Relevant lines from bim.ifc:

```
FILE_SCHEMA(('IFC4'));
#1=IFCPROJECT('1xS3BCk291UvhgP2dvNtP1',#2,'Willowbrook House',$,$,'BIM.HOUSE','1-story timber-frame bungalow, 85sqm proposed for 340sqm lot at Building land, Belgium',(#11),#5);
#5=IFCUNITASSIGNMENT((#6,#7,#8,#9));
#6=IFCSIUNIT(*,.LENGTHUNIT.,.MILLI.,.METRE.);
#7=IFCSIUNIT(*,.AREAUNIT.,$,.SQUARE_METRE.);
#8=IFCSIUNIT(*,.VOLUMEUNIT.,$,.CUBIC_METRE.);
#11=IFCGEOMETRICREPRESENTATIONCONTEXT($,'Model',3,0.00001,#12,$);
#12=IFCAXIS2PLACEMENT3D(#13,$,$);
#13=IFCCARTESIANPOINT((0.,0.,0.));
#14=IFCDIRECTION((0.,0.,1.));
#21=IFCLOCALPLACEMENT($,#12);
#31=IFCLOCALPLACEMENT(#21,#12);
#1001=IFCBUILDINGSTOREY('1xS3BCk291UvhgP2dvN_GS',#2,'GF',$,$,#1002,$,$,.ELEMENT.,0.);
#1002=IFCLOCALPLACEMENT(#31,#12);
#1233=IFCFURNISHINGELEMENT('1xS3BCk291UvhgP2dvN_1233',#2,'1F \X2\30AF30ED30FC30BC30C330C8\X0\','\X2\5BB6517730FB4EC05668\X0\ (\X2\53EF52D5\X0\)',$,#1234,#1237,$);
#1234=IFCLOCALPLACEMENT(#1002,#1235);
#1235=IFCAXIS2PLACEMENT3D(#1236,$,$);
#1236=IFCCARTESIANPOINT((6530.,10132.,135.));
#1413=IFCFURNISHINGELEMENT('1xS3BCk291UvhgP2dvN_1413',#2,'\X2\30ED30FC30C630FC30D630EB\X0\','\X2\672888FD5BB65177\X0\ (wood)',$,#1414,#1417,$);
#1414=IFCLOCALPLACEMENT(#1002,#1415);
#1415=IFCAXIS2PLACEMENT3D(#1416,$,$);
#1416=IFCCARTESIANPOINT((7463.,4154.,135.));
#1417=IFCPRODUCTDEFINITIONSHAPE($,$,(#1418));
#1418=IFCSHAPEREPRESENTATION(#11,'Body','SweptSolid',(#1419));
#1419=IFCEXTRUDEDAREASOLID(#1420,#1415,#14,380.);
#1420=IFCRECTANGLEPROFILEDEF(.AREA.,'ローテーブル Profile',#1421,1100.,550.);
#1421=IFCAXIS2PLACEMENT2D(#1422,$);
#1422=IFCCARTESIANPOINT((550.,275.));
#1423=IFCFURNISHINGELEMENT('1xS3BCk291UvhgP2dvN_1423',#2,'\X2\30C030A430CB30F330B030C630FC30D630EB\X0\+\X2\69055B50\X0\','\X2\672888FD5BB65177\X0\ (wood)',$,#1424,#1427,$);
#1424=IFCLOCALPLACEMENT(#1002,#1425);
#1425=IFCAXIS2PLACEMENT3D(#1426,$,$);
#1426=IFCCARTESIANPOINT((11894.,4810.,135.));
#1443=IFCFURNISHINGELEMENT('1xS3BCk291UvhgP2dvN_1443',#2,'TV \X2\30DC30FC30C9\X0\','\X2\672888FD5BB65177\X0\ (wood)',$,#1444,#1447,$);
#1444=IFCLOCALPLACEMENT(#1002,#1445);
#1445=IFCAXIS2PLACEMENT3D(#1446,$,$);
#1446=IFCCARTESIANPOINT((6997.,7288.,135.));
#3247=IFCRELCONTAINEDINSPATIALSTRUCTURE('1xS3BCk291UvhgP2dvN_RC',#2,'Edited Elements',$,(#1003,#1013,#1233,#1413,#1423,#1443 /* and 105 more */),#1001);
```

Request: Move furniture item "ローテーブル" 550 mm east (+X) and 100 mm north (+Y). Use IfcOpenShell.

```python
import ifcopenshell
import ifcopenshell.api.geometry
import ifcopenshell.util.placement

model = ifcopenshell.open("bim.ifc")

item = model.by_guid("1xS3BCk291UvhgP2dvN_1413")
matrix = ifcopenshell.util.placement.get_local_placement(item.ObjectPlacement)
matrix[0, 3] += 550.0
matrix[1, 3] += 100.0
ifcopenshell.api.geometry.edit_object_placement(model, product=item, matrix=matrix, is_si=False)

print(ifcopenshell.util.placement.get_local_placement(item.ObjectPlacement).round(3) + 0.0)

model.write("bim_edited.ifc")
```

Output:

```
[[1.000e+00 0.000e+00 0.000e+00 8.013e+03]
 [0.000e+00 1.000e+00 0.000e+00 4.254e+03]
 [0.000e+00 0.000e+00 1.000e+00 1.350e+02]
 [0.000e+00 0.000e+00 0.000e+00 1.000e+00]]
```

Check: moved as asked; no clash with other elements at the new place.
